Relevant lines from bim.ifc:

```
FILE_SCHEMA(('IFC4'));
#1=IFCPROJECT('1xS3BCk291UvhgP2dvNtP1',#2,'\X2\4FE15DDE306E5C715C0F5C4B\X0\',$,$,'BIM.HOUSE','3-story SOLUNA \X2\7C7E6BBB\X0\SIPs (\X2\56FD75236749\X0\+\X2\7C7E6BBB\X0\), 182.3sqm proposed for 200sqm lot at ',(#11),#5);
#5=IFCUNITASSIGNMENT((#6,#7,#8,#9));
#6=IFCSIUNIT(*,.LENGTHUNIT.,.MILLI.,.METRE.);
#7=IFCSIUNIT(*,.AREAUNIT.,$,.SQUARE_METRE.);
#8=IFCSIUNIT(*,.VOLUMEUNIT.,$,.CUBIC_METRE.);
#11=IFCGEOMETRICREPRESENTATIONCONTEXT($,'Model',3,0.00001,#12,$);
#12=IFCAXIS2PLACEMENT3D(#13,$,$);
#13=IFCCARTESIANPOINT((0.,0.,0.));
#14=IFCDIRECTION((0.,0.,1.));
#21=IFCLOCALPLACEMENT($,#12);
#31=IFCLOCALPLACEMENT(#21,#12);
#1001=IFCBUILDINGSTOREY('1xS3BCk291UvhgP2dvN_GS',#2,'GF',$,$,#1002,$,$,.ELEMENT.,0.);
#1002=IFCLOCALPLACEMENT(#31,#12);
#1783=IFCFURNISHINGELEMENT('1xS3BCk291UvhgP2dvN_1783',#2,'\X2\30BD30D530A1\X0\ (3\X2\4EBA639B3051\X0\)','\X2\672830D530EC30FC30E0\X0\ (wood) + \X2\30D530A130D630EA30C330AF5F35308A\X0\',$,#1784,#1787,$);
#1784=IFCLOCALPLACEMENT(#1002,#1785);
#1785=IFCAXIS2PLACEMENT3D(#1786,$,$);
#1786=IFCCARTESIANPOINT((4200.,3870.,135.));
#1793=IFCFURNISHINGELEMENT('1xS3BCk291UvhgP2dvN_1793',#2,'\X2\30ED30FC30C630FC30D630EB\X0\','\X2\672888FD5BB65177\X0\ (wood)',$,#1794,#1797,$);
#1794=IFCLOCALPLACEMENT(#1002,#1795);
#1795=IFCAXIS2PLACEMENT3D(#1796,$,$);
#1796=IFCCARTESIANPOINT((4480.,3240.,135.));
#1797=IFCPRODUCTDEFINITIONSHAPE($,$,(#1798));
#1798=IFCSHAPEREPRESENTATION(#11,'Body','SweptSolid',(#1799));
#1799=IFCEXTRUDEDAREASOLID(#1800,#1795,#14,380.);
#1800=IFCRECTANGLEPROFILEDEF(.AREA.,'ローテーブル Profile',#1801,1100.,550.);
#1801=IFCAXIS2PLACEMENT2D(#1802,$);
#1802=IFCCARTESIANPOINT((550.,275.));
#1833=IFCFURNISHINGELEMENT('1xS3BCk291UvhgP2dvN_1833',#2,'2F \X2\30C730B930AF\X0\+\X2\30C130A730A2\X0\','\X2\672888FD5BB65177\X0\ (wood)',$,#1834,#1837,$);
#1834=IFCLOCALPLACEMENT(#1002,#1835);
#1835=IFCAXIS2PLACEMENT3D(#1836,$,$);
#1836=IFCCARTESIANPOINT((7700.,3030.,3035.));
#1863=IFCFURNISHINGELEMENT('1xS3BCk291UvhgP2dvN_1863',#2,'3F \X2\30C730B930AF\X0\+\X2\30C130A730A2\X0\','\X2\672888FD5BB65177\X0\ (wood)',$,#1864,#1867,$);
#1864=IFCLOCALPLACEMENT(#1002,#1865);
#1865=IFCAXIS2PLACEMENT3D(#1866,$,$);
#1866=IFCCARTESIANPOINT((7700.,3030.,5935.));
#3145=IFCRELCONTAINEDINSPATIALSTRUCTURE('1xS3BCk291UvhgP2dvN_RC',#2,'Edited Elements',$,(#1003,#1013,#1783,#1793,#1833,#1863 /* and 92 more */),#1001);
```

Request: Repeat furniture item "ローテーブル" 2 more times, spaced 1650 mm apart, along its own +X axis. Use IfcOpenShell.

```python
import ifcopenshell
import ifcopenshell.api.geometry
import ifcopenshell.api.root
import ifcopenshell.util.element
import ifcopenshell.util.placement
import ifcopenshell.util.unit

model = ifcopenshell.open("bim.ifc")
unit_scale = ifcopenshell.util.unit.calculate_unit_scale(model)


def reuse_history(source, copy):
    """copy_class also copies each property set's owner history, people and application; keep the originals."""
    for rel in copy.IsDefinedBy:
        if rel.is_a("IfcRelDefinesByProperties") and (history := rel.RelatingPropertyDefinition.OwnerHistory):
            rel.RelatingPropertyDefinition.OwnerHistory = source.OwnerHistory
            ifcopenshell.util.element.remove_deep2(model, history)


source = model.by_id(1793)
base = ifcopenshell.util.placement.get_local_placement(source.ObjectPlacement)
step = base[:3, 0] * 1.65 / unit_scale

for i in range(1, 3):
    copy = ifcopenshell.api.root.copy_class(model, product=source)
    copy.Representation = ifcopenshell.util.element.copy_deep(
        model, source.Representation, exclude=["IfcGeometricRepresentationContext", "IfcRepresentationMap"]
    )
    reuse_history(source, copy)
    matrix = base.copy()
    matrix[:3, 3] += i * step
    print("added at", matrix[:3, 3].round(3) + 0.0)
    ifcopenshell.api.geometry.edit_object_placement(model, product=copy, matrix=matrix, is_si=False)

model.write("bim_v2.ifc")
```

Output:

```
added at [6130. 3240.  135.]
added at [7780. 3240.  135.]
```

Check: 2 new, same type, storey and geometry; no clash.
